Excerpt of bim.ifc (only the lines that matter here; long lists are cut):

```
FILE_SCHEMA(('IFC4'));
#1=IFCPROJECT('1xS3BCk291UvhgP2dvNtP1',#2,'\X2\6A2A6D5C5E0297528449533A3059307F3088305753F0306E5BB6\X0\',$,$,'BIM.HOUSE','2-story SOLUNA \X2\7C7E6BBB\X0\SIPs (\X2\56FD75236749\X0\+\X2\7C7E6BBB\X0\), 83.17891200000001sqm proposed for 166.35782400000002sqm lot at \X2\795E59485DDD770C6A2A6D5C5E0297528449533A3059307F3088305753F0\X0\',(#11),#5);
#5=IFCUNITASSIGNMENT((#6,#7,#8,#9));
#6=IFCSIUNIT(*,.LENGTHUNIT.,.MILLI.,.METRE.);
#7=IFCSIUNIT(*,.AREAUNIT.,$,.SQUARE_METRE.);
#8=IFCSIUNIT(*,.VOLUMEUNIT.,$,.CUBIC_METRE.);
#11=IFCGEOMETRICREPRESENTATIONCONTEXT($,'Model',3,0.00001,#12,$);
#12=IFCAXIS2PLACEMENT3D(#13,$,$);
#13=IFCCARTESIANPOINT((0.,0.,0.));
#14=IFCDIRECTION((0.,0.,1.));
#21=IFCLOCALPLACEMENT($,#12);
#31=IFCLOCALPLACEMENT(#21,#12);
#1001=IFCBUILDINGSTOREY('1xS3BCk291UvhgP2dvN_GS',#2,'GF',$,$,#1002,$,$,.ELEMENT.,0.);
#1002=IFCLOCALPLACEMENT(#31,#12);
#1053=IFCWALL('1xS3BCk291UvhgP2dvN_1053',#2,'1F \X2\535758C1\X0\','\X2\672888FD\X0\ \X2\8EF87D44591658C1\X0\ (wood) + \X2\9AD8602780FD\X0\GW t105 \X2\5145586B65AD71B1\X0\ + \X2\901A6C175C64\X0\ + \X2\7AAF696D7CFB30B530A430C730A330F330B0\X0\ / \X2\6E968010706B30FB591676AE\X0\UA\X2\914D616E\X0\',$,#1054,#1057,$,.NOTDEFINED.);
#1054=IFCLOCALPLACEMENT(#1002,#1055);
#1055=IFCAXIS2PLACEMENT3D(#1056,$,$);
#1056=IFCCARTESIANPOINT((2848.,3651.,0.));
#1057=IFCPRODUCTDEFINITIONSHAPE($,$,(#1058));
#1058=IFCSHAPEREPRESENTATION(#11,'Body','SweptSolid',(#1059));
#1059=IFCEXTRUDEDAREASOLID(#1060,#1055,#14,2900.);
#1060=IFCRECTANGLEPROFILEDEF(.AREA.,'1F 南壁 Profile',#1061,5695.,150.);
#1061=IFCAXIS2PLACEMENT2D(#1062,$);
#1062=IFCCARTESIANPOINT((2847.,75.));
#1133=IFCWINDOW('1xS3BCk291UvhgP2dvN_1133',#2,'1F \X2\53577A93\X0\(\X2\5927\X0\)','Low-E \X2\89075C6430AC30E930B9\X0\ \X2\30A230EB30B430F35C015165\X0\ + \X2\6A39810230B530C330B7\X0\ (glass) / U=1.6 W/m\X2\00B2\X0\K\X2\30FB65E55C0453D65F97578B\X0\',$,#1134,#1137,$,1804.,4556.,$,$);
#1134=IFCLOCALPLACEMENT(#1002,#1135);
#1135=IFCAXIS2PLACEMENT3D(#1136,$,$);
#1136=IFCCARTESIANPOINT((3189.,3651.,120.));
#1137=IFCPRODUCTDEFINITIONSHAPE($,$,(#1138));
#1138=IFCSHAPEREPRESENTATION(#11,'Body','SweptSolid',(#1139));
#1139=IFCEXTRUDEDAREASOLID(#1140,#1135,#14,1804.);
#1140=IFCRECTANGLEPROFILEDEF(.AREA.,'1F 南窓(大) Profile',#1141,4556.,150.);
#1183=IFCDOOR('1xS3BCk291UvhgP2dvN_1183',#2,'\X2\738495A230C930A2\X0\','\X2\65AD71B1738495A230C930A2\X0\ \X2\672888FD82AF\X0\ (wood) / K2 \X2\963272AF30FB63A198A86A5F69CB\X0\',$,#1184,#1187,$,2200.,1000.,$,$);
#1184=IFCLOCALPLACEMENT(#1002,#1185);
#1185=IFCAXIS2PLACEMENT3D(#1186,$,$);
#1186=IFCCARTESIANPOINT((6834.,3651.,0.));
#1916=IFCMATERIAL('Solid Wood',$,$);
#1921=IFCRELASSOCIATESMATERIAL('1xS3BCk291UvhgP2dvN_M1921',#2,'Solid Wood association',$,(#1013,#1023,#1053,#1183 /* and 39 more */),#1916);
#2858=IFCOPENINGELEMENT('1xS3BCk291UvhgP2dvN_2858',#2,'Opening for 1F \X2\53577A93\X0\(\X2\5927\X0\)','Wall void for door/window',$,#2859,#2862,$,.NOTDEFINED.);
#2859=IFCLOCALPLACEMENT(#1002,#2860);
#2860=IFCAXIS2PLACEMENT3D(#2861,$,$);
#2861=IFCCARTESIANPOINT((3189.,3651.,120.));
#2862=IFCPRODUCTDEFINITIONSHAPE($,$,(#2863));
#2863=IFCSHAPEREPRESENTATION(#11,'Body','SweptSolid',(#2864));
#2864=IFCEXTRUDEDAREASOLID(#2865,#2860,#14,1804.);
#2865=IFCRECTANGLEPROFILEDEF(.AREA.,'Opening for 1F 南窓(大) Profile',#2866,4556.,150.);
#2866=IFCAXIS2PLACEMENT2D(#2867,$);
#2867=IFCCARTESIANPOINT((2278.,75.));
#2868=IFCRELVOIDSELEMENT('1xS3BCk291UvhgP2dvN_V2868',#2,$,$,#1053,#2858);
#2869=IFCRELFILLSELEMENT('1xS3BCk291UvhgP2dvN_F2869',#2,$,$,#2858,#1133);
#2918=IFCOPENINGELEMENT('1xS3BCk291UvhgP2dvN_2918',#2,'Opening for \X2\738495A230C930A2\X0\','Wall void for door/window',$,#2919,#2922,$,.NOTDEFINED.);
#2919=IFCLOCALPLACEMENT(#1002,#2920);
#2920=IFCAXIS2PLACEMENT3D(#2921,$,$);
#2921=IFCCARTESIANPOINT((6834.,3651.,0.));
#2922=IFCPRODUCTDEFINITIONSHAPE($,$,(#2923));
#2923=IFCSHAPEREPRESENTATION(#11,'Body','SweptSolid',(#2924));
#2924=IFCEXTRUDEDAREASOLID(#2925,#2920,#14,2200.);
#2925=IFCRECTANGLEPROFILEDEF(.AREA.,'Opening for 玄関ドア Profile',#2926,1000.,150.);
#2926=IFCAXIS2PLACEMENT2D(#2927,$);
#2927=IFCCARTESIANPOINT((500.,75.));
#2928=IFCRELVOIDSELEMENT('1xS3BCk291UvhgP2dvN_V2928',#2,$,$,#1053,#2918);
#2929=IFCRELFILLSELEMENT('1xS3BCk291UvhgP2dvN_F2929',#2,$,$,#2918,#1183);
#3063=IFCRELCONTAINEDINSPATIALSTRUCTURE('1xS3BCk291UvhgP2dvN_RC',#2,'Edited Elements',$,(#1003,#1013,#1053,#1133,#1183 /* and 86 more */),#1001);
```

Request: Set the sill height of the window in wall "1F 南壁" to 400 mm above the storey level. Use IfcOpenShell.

```python
import numpy as np
import ifcopenshell
import ifcopenshell.api.geometry
import ifcopenshell.geom
import ifcopenshell.util.element
import ifcopenshell.util.placement
import ifcopenshell.util.shape
import ifcopenshell.util.unit

model = ifcopenshell.open("bim.ifc")
unit_scale = ifcopenshell.util.unit.calculate_unit_scale(model)

window = model.by_guid("1xS3BCk291UvhgP2dvN_1133")
opening = window.FillsVoids[0].RelatingOpeningElement
storey = ifcopenshell.util.element.get_container(window, ifc_class="IfcBuildingStorey")
level = ifcopenshell.util.placement.get_local_placement(storey.ObjectPlacement)[2, 3]

# The opening's origin need not be at the sill, so measure its lowest point.
shape = ifcopenshell.geom.create_shape(ifcopenshell.geom.settings(), opening)
bottom = ifcopenshell.util.shape.get_shape_bottom_elevation(shape, shape.geometry) / unit_scale
dz = level + 0.4 / unit_scale - bottom

shift = np.array([0.0, 0.0, dz])
# The window is not placed relative to its opening, so move both.
for product in (opening, window):
    matrix = ifcopenshell.util.placement.get_local_placement(product.ObjectPlacement)
    matrix[:3, 3] += shift
    ifcopenshell.api.geometry.edit_object_placement(model, product=product, matrix=matrix, is_si=False)

print(f"moved by {dz * unit_scale:+.3f} m")

model.write("bim-out.ifc")
```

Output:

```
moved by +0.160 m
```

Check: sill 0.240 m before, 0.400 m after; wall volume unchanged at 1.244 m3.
